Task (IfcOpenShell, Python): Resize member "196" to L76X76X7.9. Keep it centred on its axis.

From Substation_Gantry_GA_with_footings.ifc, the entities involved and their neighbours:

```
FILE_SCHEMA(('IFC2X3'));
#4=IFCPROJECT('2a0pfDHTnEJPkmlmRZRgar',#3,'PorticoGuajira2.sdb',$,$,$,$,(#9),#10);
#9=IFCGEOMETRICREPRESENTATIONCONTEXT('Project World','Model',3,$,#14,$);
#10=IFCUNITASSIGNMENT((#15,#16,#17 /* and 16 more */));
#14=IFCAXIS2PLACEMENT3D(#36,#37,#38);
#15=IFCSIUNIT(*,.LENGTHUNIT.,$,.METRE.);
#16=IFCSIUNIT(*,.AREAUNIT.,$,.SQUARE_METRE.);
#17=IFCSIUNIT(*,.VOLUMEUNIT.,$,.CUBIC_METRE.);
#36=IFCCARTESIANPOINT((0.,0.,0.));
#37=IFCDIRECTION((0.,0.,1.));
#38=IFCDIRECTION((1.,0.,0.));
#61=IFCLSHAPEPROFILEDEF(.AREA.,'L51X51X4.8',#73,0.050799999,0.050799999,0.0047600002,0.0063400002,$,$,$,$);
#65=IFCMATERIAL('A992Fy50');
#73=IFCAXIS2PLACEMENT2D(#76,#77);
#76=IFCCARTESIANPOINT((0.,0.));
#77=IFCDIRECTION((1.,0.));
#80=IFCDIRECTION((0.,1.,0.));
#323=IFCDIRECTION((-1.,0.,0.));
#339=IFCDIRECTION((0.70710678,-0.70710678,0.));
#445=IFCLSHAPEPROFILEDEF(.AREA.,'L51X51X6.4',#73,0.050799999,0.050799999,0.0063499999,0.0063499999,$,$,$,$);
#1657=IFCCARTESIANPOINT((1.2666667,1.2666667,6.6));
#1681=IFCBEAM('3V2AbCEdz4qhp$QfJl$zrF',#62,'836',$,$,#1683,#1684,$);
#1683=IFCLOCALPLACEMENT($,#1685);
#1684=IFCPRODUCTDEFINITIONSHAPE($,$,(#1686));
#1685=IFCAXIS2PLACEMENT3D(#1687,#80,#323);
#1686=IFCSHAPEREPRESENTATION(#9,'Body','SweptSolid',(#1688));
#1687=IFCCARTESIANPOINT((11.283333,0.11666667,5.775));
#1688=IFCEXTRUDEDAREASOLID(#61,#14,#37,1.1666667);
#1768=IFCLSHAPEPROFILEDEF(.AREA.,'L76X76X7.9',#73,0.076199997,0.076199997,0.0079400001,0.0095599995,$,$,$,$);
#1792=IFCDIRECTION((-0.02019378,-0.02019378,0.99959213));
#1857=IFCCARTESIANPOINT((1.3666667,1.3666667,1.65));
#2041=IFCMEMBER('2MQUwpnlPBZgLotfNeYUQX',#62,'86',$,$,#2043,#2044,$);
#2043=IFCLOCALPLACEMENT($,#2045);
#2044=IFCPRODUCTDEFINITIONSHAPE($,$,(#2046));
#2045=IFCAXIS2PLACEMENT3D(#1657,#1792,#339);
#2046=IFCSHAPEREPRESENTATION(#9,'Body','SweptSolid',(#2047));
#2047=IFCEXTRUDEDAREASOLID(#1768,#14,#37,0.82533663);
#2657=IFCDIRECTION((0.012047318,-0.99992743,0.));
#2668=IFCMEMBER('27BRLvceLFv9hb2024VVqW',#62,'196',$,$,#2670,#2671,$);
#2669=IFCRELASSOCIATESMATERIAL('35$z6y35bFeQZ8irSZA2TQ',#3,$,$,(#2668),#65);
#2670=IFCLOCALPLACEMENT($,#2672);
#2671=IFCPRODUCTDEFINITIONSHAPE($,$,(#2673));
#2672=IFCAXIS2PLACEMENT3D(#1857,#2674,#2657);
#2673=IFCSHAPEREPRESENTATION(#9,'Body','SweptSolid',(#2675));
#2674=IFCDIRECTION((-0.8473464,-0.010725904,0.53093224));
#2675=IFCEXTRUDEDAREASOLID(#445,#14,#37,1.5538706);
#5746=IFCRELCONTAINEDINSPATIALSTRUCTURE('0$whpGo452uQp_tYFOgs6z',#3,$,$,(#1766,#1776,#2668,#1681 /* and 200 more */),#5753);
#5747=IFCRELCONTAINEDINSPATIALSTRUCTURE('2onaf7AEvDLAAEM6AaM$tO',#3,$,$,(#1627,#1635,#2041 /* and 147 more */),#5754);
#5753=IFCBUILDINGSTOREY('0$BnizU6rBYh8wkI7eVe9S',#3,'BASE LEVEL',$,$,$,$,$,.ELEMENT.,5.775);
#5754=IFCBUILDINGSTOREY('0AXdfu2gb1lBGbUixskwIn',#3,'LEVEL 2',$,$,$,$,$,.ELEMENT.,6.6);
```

```python
import ifcopenshell
import ifcopenshell.util.element

model = ifcopenshell.open("Substation_Gantry_GA_with_footings.ifc")

member = model.by_guid("27BRLvceLFv9hb2024VVqW")
source = next(p for p in model.by_type("IfcLShapeProfileDef") if p.ProfileName == "L76X76X7.9")

body = next(r for r in member.Representation.Representations if r.RepresentationIdentifier == "Body")
solid = body.Items[0]
old_profile = solid.SweptArea

# Copy the section's sizes but keep this member's own profile position.
profile = ifcopenshell.util.element.copy(model, source)
profile.Position = old_profile.Position
solid.SweptArea = profile
if not model.get_total_inverses(old_profile):
    ifcopenshell.util.element.remove_deep2(model, old_profile)

print(solid.SweptArea)

model.write("Substation_Gantry_GA_with_footings_edited.ifc")
```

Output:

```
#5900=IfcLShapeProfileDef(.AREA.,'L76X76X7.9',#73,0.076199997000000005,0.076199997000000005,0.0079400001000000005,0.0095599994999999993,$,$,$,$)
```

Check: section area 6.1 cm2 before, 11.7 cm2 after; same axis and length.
